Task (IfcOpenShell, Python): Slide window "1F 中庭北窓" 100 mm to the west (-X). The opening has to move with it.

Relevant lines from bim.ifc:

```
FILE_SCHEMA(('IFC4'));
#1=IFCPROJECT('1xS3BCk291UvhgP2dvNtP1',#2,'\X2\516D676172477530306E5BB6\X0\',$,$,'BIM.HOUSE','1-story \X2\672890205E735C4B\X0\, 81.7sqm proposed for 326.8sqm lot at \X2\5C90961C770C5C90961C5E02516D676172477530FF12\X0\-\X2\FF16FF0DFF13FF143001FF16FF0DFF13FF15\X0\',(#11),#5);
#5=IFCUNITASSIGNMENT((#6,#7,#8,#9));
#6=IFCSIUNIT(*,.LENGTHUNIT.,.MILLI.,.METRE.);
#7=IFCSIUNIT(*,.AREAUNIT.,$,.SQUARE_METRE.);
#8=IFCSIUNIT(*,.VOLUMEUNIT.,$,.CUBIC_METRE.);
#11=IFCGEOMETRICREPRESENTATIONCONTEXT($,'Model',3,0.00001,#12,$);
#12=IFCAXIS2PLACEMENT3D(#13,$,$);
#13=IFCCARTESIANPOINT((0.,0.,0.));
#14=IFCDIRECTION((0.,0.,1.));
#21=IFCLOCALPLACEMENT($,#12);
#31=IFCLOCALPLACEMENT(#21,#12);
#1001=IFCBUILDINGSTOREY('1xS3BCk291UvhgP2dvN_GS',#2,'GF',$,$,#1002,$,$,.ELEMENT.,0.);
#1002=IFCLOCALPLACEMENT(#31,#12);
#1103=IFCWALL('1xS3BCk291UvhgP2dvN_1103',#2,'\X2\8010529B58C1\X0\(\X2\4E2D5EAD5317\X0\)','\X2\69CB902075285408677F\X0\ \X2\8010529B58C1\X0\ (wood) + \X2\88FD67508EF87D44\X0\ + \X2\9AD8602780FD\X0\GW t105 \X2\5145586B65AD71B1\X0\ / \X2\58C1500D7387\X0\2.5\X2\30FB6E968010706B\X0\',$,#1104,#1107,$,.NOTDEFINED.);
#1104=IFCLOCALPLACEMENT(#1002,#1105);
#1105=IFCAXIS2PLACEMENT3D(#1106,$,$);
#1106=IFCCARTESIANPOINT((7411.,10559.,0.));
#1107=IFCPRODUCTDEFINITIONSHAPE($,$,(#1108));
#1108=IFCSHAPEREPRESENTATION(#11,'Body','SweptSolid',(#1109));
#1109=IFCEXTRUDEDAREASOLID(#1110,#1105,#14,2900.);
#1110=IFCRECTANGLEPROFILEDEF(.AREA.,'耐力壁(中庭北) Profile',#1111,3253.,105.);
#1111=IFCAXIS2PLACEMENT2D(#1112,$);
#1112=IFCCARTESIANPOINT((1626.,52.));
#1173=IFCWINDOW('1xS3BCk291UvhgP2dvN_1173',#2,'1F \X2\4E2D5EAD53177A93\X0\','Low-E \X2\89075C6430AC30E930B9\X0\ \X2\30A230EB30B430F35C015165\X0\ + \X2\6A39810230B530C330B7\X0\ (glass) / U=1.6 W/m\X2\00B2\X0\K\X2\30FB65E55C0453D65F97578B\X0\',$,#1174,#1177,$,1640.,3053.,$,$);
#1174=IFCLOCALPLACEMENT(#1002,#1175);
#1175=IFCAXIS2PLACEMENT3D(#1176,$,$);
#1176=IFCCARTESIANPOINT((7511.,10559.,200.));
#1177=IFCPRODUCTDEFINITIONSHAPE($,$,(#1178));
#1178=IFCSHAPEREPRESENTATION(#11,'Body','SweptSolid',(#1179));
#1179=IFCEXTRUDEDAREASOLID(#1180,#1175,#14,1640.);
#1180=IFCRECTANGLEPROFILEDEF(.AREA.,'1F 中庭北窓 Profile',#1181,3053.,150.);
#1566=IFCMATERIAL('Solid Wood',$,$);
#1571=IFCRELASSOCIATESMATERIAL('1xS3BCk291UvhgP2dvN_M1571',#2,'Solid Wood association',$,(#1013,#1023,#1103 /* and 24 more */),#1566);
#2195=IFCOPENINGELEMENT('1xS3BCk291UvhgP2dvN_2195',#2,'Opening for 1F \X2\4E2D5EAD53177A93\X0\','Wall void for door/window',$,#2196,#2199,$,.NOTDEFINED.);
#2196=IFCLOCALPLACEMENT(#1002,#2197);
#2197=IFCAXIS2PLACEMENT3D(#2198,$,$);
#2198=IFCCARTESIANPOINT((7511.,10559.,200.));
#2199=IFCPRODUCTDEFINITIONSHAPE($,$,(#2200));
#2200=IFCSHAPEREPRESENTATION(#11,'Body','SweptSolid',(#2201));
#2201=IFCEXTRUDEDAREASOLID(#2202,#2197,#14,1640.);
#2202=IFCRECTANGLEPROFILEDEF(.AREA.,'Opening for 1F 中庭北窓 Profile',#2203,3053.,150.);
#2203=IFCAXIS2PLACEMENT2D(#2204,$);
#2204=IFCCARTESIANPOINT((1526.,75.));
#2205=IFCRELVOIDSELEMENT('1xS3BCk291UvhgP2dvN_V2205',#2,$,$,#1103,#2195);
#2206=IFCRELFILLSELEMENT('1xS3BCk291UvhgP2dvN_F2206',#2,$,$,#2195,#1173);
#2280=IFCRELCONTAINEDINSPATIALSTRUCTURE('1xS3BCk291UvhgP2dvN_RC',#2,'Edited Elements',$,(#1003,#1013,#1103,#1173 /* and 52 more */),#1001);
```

```python
import ifcopenshell
import ifcopenshell.api.geometry
import ifcopenshell.util.placement
import ifcopenshell.util.unit

model = ifcopenshell.open("bim.ifc")
unit_scale = ifcopenshell.util.unit.calculate_unit_scale(model)

window = model.by_guid("1xS3BCk291UvhgP2dvN_1173")
opening = window.FillsVoids[0].RelatingOpeningElement
wall = opening.VoidsElements[0].RelatingBuildingElement

wall_matrix = ifcopenshell.util.placement.get_local_placement(wall.ObjectPlacement)
shift = wall_matrix[:3, 0] * -0.1 / unit_scale
before = ifcopenshell.util.placement.get_local_placement(window.ObjectPlacement)[:3, 3].copy()

# The window is not placed relative to its opening, so move both.
for product in (opening, window):
    matrix = ifcopenshell.util.placement.get_local_placement(product.ObjectPlacement)
    matrix[:3, 3] += shift
    ifcopenshell.api.geometry.edit_object_placement(model, product=product, matrix=matrix, is_si=False)

after = ifcopenshell.util.placement.get_local_placement(window.ObjectPlacement)[:3, 3]
print("window moved by", (after - before).round(3) + 0.0)

model.write("bim_v2.ifc")
```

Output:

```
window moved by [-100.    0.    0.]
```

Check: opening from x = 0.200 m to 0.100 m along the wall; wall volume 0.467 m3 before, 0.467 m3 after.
